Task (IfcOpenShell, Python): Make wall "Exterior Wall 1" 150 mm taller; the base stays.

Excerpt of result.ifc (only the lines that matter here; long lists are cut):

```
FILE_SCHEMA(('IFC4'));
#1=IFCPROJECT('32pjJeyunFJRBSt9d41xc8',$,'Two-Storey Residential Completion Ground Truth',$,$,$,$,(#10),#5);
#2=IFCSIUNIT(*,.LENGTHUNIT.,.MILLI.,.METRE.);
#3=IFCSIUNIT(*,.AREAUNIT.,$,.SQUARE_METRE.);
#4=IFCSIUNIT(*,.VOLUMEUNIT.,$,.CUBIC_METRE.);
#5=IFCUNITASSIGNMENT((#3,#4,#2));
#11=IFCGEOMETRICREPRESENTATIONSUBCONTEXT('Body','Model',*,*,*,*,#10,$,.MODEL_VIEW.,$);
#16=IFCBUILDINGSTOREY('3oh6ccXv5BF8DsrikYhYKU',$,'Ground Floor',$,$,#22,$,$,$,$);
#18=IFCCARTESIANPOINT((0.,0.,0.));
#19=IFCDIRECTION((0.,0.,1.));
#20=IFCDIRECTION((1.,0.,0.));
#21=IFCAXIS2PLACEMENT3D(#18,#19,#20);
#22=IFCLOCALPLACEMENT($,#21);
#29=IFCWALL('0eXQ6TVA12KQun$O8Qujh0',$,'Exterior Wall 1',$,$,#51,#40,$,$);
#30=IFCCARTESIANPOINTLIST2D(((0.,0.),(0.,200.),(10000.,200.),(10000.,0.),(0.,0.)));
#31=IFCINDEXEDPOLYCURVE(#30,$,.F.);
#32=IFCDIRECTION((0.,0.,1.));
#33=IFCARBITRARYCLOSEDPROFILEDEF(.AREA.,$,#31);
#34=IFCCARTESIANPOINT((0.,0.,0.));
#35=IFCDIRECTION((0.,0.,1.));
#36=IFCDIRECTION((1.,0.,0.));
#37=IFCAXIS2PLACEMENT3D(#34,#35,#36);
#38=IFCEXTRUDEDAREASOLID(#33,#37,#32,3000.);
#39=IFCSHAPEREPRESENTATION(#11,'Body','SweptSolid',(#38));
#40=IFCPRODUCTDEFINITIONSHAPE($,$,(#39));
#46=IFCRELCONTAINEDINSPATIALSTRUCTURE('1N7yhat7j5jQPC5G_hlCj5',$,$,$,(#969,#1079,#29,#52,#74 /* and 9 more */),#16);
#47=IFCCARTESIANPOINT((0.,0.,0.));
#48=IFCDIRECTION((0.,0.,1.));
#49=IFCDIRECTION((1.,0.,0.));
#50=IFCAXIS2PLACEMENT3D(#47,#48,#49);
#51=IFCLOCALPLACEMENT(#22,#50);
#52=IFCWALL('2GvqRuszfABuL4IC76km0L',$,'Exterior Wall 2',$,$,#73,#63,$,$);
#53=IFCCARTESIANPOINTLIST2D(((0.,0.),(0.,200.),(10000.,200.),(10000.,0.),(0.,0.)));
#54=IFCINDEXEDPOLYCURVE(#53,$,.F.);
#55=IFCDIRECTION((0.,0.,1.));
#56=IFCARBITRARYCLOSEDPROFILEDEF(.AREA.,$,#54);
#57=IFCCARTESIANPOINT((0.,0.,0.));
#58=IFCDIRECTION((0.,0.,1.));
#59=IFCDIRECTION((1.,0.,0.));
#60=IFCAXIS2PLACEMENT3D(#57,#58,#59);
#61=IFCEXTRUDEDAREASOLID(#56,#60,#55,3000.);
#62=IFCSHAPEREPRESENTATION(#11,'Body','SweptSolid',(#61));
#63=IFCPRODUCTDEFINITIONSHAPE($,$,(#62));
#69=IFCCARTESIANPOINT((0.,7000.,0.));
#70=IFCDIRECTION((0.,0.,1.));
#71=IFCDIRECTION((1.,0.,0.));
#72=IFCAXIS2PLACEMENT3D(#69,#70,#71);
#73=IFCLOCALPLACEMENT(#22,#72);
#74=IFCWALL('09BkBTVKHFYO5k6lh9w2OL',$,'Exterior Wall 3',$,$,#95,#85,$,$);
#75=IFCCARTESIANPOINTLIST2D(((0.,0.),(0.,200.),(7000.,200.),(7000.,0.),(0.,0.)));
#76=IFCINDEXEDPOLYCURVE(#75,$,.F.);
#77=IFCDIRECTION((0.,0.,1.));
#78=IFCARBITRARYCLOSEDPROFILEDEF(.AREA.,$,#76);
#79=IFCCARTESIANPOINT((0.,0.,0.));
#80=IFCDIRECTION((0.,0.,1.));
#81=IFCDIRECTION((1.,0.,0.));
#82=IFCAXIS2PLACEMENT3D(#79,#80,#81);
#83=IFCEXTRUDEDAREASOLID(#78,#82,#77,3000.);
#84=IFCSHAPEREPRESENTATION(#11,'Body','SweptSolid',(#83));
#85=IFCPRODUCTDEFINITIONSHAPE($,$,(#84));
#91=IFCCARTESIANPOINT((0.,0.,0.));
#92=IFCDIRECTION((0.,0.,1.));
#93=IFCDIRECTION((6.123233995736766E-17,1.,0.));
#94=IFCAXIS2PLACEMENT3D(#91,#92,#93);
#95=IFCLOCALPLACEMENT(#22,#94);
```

```python
import ifcopenshell
import ifcopenshell.geom
import ifcopenshell.util.representation
import ifcopenshell.util.shape

model = ifcopenshell.open("result.ifc")
settings = ifcopenshell.geom.settings()


def volume(element):
    """Net volume in cubic metres, openings subtracted."""
    shape = ifcopenshell.geom.create_shape(settings, element)
    return ifcopenshell.util.shape.get_volume(shape.geometry)


wall = model.by_guid("0eXQ6TVA12KQun$O8Qujh0")
before = volume(wall)

body = ifcopenshell.util.representation.get_representation(wall, "Model", "Body")
solid = body.Items[0]
old_height = solid.Depth
solid.Depth += 150.0
after = volume(wall)

print(f"height {old_height:g} -> {solid.Depth:g}, volume {before:.3f} -> {after:.3f} m3")

model.write("result_v2.ifc")
```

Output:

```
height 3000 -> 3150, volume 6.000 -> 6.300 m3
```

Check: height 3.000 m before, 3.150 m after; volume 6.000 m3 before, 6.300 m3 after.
